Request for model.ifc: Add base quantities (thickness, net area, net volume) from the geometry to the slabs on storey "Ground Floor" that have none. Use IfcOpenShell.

First a look at what the model holds.

```python
import ifcopenshell
import ifcopenshell.util.element
import ifcopenshell.util.unit

model = ifcopenshell.open("model.ifc")
print(model.schema)
for unit_type in ("LENGTHUNIT", "AREAUNIT", "VOLUMEUNIT"):
    print(unit_type, ifcopenshell.util.unit.calculate_unit_scale(model, unit_type))
storey = next(s for s in model.by_type("IfcBuildingStorey") if s.Name == "Ground Floor")
slabs = [e for e in ifcopenshell.util.element.get_decomposition(storey) if e.is_a("IfcSlab")]
for e in sorted(slabs, key=lambda e: e.id()):
    print(e.id(), e.is_a(), e.Name, list(ifcopenshell.util.element.get_psets(e, qtos_only=True)), sep=" | ")
```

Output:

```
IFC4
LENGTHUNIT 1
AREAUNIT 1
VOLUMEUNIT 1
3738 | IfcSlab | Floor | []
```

```python
import ifcopenshell
import ifcopenshell.api.pset
import ifcopenshell.geom
import ifcopenshell.util.element
import ifcopenshell.util.shape
import ifcopenshell.util.unit

model = ifcopenshell.open("model.ifc")
unit_scale = ifcopenshell.util.unit.calculate_unit_scale(model)
area_scale = ifcopenshell.util.unit.calculate_unit_scale(model, "AREAUNIT")
volume_scale = ifcopenshell.util.unit.calculate_unit_scale(model, "VOLUMEUNIT")
settings = ifcopenshell.geom.settings()

storey = next(s for s in model.by_type("IfcBuildingStorey") if s.Name == "Ground Floor")
slabs = [e for e in ifcopenshell.util.element.get_decomposition(storey) if e.is_a("IfcSlab")]

for e in sorted(slabs, key=lambda e: e.id()):
    if ifcopenshell.util.element.get_psets(e, qtos_only=True, should_inherit=False):
        continue
    # Geometry comes back in metres, in the element's own axes.
    shape = ifcopenshell.geom.create_shape(settings, e)
    values = {
        "Width": ifcopenshell.util.shape.get_z(shape.geometry) / unit_scale,
        "NetArea": ifcopenshell.util.shape.get_footprint_area(shape.geometry) / area_scale,
        "NetVolume": ifcopenshell.util.shape.get_volume(shape.geometry) / volume_scale,
    }
    qto = ifcopenshell.api.pset.add_qto(model, product=e, name="Qto_SlabBaseQuantities")
    ifcopenshell.api.pset.edit_qto(model, qto=qto, properties=values)
    print(e.id(), {k: round(v, 3) for k, v in values.items()})

model.write("model-out.ifc")
```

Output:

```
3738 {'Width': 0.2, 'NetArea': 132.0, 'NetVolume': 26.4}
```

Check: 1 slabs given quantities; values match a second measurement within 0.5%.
